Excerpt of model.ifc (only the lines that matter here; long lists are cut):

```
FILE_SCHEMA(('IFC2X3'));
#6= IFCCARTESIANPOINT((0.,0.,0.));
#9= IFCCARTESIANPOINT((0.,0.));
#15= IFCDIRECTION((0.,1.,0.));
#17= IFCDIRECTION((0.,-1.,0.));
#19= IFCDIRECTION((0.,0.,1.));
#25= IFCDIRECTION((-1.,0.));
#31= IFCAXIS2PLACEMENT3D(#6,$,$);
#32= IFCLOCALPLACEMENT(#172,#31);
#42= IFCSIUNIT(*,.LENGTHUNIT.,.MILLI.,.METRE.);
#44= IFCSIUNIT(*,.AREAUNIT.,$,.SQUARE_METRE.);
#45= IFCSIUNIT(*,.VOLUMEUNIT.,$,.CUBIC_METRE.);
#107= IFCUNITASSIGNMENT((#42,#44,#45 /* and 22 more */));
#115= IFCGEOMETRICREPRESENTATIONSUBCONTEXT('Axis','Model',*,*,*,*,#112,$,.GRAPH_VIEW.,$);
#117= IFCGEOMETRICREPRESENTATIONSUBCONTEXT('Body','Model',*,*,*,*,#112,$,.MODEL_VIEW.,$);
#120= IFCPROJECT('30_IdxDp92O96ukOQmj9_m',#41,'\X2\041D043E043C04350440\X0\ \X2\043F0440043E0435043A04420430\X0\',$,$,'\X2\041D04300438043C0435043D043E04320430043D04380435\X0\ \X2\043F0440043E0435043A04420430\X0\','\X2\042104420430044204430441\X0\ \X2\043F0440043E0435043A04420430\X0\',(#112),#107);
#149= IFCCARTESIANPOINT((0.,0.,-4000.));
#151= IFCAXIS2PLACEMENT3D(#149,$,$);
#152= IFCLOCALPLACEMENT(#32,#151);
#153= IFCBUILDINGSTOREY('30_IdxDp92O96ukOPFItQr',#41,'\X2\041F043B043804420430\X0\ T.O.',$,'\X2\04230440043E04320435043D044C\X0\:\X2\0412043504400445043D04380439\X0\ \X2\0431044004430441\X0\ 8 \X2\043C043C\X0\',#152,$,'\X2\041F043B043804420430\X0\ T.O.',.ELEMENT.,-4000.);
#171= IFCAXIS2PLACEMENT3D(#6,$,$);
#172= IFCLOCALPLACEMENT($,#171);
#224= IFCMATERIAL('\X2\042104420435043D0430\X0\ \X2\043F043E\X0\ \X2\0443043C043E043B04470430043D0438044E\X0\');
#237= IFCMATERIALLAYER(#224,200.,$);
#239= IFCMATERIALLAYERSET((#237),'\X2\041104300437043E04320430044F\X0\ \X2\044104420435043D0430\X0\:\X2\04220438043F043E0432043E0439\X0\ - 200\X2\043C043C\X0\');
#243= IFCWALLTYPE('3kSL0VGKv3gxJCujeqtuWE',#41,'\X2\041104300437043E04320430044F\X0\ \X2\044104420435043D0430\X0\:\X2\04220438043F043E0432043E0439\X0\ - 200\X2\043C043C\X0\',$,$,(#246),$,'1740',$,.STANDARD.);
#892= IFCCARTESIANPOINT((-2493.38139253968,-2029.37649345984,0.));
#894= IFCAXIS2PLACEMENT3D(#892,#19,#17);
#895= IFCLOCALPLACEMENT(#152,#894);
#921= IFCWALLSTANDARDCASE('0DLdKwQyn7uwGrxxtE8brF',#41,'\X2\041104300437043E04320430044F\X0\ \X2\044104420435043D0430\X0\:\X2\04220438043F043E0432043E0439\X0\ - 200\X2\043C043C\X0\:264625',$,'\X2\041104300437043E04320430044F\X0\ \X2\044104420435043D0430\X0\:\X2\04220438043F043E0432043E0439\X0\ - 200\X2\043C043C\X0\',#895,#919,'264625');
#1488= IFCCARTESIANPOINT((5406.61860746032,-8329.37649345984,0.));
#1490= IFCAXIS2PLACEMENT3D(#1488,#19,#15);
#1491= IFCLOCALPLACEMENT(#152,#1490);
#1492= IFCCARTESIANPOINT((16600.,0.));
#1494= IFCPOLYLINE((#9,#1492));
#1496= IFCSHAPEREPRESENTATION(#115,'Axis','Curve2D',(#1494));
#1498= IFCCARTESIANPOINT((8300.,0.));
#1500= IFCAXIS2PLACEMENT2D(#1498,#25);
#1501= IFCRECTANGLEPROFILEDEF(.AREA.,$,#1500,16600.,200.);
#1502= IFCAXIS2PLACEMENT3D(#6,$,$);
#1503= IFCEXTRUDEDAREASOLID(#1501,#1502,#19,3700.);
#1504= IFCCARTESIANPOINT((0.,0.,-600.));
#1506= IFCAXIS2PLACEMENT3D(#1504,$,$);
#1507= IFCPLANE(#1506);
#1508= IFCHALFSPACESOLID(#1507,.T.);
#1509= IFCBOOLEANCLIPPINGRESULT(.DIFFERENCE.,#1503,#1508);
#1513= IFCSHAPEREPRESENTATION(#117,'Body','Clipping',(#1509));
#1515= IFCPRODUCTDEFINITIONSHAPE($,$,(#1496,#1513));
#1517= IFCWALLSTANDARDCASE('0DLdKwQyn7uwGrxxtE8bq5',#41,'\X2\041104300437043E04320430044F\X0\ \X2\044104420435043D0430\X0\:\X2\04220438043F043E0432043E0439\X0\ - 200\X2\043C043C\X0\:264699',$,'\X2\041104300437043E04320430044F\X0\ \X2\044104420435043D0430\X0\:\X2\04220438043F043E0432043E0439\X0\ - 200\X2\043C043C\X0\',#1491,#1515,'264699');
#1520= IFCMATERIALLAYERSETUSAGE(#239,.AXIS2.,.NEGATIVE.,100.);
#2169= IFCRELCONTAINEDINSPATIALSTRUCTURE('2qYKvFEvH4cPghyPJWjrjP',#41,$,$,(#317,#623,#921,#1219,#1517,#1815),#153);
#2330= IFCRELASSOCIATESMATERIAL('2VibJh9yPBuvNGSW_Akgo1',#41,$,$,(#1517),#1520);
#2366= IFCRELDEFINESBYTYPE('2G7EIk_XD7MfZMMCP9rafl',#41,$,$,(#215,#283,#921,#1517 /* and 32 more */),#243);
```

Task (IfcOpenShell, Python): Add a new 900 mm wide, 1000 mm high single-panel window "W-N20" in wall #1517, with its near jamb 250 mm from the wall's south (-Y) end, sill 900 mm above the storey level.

```python
import numpy as np
import ifcopenshell
import ifcopenshell.api.feature
import ifcopenshell.api.geometry
import ifcopenshell.api.root
import ifcopenshell.api.spatial
import ifcopenshell.api.type
import ifcopenshell.geom
import ifcopenshell.util.element
import ifcopenshell.util.placement
import ifcopenshell.util.representation
import ifcopenshell.util.shape
import ifcopenshell.util.unit

model = ifcopenshell.open("model.ifc")
unit_scale = ifcopenshell.util.unit.calculate_unit_scale(model)
settings = ifcopenshell.geom.settings()


def volume(element):
    """Net volume in cubic metres, openings subtracted."""
    shape = ifcopenshell.geom.create_shape(settings, element)
    return ifcopenshell.util.shape.get_volume(shape.geometry)


wall = model.by_guid("0DLdKwQyn7uwGrxxtE8bq5")
storey = ifcopenshell.util.element.get_container(wall, ifc_class="IfcBuildingStorey")
context = ifcopenshell.util.representation.get_context(model, "Model", "Body", "MODEL_VIEW")
before = volume(wall)

width, height, from_end, sill = 0.9, 1, 0.25, 0.9  # metres

# The wall runs along its own X axis, and the end named is its -X end.
wall_shape = ifcopenshell.geom.create_shape(settings, wall)
x, y, z = ifcopenshell.util.shape.get_vertices(wall_shape.geometry).T
start = x.min() + from_end
face, thickness = float(y.min()), float(y.max() - y.min())
wall_matrix = ifcopenshell.util.placement.get_local_placement(wall.ObjectPlacement)
level = ifcopenshell.util.placement.get_local_placement(storey.ObjectPlacement)[2, 3]


def in_wall(x, y):
    """Placement at x, y metres in the wall's axes, at sill height."""
    matrix = wall_matrix.copy()
    matrix[:, 3] = wall_matrix @ np.array([x / unit_scale, y / unit_scale, 0.0, 1.0])
    matrix[2, 3] = level + sill / unit_scale
    return matrix


# Opening: a box that overshoots both wall faces by 50 mm.
opening = ifcopenshell.api.root.create_entity(model, ifc_class="IfcOpeningElement")
box = ifcopenshell.api.geometry.add_wall_representation(
    model, context=context, length=width, height=height, thickness=thickness + 0.1
)
ifcopenshell.api.geometry.assign_representation(model, product=opening, representation=box)
ifcopenshell.api.geometry.edit_object_placement(model, product=opening, matrix=in_wall(start, face - 0.05), is_si=False)
ifcopenshell.api.feature.add_feature(model, feature=opening, element=wall)

window = ifcopenshell.api.root.create_entity(model, ifc_class="IfcWindow", name="W-N20")
window.OverallWidth, window.OverallHeight = width / unit_scale, height / unit_scale
body = ifcopenshell.api.geometry.add_window_representation(
    model,
    context=context,
    overall_width=window.OverallWidth,
    overall_height=window.OverallHeight,
    partition_type="SINGLE_PANEL",
)
ifcopenshell.api.geometry.assign_representation(model, product=window, representation=body)
ifcopenshell.api.spatial.assign_container(model, products=[window], relating_structure=storey)
fills = ifcopenshell.api.feature.add_filling(model, opening=opening, element=window)
fills.OwnerHistory = window.OwnerHistory  # required in IFC2X3

# IFC2X3 keeps the operation on the window style.
style = ifcopenshell.api.root.create_entity(model, ifc_class="IfcWindowStyle", name="W-N20")
style.OperationType, style.ConstructionType = "SINGLE_PANEL", "NOTDEFINED"
style.ParameterTakesPrecedence = style.Sizeable = False
ifcopenshell.api.type.assign_type(model, related_objects=[window], relating_type=style)

# Centre the window in the wall's thickness.
ifcopenshell.api.geometry.edit_object_placement(model, product=window, matrix=in_wall(start, face), is_si=False)
window_shape = ifcopenshell.geom.create_shape(settings, window)
depth = ifcopenshell.util.shape.get_vertices(window_shape.geometry)[:, 1]
offset = face + thickness / 2 - (depth.min() + depth.max()) / 2
ifcopenshell.api.geometry.edit_object_placement(model, product=window, matrix=in_wall(start, offset), is_si=False)

after = volume(wall)

print(f"wall volume {before:.3f} -> {after:.3f} m3")

model.write("model-out.ifc")
```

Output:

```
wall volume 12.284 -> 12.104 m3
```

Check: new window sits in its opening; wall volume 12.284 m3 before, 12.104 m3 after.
